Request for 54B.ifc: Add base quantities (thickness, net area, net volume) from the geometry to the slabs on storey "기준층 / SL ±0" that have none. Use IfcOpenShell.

First a look at what the model holds.

```python
import ifcopenshell
import ifcopenshell.util.element
import ifcopenshell.util.unit

model = ifcopenshell.open("54B.ifc")
print(model.schema)
for unit_type in ("LENGTHUNIT", "AREAUNIT", "VOLUMEUNIT"):
    print(unit_type, ifcopenshell.util.unit.calculate_unit_scale(model, unit_type))
storey = next(s for s in model.by_type("IfcBuildingStorey") if s.Name == "기준층 / SL ±0")
slabs = [e for e in ifcopenshell.util.element.get_decomposition(storey) if e.is_a("IfcSlab")]
for e in sorted(slabs, key=lambda e: e.id()):
    print(e.id(), e.is_a(), e.Name, list(ifcopenshell.util.element.get_psets(e, qtos_only=True)), sep=" | ")
```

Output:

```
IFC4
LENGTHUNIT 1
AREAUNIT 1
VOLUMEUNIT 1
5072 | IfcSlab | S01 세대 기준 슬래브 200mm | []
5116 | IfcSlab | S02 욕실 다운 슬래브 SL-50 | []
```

```python
import ifcopenshell
import ifcopenshell.api.pset
import ifcopenshell.geom
import ifcopenshell.util.element
import ifcopenshell.util.shape
import ifcopenshell.util.unit

model = ifcopenshell.open("54B.ifc")
unit_scale = ifcopenshell.util.unit.calculate_unit_scale(model)
area_scale = ifcopenshell.util.unit.calculate_unit_scale(model, "AREAUNIT")
volume_scale = ifcopenshell.util.unit.calculate_unit_scale(model, "VOLUMEUNIT")
settings = ifcopenshell.geom.settings()

storey = next(s for s in model.by_type("IfcBuildingStorey") if s.Name == "기준층 / SL ±0")
slabs = [e for e in ifcopenshell.util.element.get_decomposition(storey) if e.is_a("IfcSlab")]

for e in sorted(slabs, key=lambda e: e.id()):
    if ifcopenshell.util.element.get_psets(e, qtos_only=True, should_inherit=False):
        continue
    # Geometry comes back in metres, in the element's own axes.
    shape = ifcopenshell.geom.create_shape(settings, e)
    values = {
        "Width": ifcopenshell.util.shape.get_z(shape.geometry) / unit_scale,
        "NetArea": ifcopenshell.util.shape.get_footprint_area(shape.geometry) / area_scale,
        "NetVolume": ifcopenshell.util.shape.get_volume(shape.geometry) / volume_scale,
    }
    qto = ifcopenshell.api.pset.add_qto(model, product=e, name="Qto_SlabBaseQuantities")
    ifcopenshell.api.pset.edit_qto(model, qto=qto, properties=values)
    print(e.id(), {k: round(v, 3) for k, v in values.items()})

model.write("54B_rev.ifc")
```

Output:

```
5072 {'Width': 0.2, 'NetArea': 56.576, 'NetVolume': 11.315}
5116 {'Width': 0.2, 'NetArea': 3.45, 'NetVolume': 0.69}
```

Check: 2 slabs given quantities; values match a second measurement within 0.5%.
